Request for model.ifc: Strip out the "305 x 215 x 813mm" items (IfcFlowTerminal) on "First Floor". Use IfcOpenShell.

First a look at what the model holds.

```python
import ifcopenshell
import ifcopenshell.util.element

model = ifcopenshell.open("model.ifc")
print(model.schema)
storey = next(s for s in model.by_type("IfcBuildingStorey") if s.Name == "First Floor")
terminals = [e for e in ifcopenshell.util.element.get_decomposition(storey) if e.is_a("IfcFlowTerminal")]
seen = {}
for e in terminals:
    element_type = ifcopenshell.util.element.get_type(e)
    name = element_type.Name if element_type not in (None, e) else None
    seen[name] = seen.get(name, 0) + 1
for name, count in sorted(seen.items(), key=str):
    print(count, "x", name)
```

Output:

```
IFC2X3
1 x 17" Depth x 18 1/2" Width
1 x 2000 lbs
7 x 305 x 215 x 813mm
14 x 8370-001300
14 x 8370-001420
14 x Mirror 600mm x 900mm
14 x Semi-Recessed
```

```python
import ifcopenshell
import ifcopenshell.api.root
import ifcopenshell.util.element

model = ifcopenshell.open("model.ifc")

storey = next(s for s in model.by_type("IfcBuildingStorey") if s.Name == "First Floor")
terminals = [e for e in ifcopenshell.util.element.get_decomposition(storey) if e.is_a("IfcFlowTerminal")]
targets = [e for e in terminals if (t := ifcopenshell.util.element.get_type(e)) not in (None, e) and t.Name == "305 x 215 x 813mm"]

for e in targets:
    ifcopenshell.api.root.remove_product(model, product=e)
print(len(targets), "removed")

model.write("model-out.ifc")
```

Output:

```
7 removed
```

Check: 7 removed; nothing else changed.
